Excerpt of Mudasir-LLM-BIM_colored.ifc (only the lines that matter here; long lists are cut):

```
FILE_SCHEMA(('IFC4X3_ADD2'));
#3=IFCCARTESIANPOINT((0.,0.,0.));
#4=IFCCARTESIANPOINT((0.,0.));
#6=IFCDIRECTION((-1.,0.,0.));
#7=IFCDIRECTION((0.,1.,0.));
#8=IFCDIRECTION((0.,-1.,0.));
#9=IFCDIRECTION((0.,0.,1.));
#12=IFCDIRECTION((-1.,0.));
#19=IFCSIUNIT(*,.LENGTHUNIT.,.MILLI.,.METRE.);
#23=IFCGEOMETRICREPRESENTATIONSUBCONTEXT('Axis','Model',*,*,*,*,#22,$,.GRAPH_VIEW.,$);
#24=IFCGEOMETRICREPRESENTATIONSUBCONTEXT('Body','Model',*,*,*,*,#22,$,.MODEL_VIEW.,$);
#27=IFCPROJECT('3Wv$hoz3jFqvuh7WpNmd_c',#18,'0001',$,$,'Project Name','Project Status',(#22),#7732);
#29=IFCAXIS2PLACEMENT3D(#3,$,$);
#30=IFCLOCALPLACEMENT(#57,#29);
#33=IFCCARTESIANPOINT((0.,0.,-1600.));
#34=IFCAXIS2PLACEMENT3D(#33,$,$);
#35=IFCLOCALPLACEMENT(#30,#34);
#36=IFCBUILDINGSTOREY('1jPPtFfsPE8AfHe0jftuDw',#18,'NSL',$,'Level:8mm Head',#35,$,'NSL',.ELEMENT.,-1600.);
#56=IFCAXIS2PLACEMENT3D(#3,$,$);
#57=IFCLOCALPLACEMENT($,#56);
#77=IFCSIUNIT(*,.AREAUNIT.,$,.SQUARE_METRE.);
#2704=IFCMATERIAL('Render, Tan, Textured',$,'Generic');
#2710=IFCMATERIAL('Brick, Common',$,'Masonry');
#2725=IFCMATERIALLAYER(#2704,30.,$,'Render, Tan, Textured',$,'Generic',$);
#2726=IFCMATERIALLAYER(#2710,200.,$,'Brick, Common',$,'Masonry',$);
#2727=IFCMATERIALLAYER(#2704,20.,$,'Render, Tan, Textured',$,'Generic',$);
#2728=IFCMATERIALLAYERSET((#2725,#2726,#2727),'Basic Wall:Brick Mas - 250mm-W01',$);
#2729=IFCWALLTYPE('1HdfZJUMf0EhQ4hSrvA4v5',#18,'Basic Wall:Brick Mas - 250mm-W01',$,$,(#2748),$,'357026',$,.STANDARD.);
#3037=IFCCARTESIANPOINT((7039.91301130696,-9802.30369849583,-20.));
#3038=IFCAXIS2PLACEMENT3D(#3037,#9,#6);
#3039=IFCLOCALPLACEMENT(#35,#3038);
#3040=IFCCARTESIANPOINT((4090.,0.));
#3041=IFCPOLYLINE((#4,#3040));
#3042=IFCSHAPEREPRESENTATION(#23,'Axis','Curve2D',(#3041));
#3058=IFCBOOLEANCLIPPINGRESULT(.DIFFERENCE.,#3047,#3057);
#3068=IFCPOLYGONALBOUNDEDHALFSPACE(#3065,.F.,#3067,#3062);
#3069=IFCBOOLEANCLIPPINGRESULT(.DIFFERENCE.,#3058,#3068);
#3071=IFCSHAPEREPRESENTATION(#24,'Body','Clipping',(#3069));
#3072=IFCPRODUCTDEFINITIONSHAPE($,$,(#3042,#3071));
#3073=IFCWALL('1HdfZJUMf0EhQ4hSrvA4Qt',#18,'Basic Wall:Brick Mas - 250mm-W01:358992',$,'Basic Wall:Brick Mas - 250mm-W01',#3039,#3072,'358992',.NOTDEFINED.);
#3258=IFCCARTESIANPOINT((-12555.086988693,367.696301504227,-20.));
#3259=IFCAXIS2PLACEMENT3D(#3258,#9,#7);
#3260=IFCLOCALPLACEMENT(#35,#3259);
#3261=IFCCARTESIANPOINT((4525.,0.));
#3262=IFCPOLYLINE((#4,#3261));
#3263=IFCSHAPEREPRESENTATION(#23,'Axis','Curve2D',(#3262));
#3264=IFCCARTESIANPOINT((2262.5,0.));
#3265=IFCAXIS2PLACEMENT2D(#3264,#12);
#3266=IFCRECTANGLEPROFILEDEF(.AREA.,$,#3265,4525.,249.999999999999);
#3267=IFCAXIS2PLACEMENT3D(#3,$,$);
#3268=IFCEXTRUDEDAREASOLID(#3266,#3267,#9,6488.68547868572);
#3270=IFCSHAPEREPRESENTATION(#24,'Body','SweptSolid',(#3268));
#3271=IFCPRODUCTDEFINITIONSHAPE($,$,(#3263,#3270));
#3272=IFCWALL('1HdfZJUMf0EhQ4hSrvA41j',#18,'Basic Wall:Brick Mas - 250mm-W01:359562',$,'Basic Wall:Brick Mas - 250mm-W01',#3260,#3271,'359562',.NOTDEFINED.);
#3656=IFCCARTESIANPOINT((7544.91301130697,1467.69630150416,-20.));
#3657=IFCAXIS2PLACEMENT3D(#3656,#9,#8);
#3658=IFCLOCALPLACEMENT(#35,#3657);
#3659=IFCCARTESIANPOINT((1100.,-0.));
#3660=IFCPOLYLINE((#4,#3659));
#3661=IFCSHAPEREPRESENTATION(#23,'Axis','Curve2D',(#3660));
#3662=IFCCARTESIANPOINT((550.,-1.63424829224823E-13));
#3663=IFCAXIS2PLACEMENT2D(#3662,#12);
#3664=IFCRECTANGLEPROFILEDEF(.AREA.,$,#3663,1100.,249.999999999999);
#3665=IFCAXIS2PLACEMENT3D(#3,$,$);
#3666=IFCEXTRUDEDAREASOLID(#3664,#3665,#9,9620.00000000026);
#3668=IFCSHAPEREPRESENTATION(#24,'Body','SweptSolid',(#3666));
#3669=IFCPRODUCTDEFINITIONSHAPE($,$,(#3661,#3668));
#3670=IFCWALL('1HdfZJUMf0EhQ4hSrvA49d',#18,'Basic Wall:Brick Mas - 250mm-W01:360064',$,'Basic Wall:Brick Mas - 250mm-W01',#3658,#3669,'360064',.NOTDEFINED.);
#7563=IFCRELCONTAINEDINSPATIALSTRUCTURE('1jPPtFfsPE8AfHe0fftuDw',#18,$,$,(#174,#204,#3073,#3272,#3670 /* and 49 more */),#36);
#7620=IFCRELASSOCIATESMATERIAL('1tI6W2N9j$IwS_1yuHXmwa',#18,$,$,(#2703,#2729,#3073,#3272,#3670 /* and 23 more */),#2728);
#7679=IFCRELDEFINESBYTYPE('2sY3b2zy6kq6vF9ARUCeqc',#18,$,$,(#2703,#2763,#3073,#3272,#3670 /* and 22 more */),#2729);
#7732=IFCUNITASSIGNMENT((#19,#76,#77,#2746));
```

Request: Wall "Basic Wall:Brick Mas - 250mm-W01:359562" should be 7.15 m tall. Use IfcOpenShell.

```python
import ifcopenshell
import ifcopenshell.geom
import ifcopenshell.util.representation
import ifcopenshell.util.shape
import ifcopenshell.util.unit

model = ifcopenshell.open("Mudasir-LLM-BIM_colored.ifc")
unit_scale = ifcopenshell.util.unit.calculate_unit_scale(model)
settings = ifcopenshell.geom.settings()


def volume(element):
    """Net volume in cubic metres, openings subtracted."""
    shape = ifcopenshell.geom.create_shape(settings, element)
    return ifcopenshell.util.shape.get_volume(shape.geometry)


wall = model.by_guid("1HdfZJUMf0EhQ4hSrvA41j")
before = volume(wall)

body = ifcopenshell.util.representation.get_representation(wall, "Model", "Body")
solid = body.Items[0]
old_height = solid.Depth
solid.Depth = 7.15 / unit_scale
after = volume(wall)

print(f"height {old_height:g} -> {solid.Depth:g}, volume {before:.3f} -> {after:.3f} m3")

model.write("Mudasir-LLM-BIM_colored_edited.ifc")
```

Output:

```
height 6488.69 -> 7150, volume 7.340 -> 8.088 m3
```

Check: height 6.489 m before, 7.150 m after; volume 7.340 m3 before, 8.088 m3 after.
